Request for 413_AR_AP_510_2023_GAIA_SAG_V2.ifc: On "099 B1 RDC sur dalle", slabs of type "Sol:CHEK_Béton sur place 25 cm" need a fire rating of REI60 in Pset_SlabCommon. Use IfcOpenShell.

First a look at what the model holds.

```python
import ifcopenshell
import ifcopenshell.util.element

model = ifcopenshell.open("413_AR_AP_510_2023_GAIA_SAG_V2.ifc")
print(model.schema)
storey = next(s for s in model.by_type("IfcBuildingStorey") if s.Name == "099 B1 RDC sur dalle")
slabs = [e for e in ifcopenshell.util.element.get_decomposition(storey) if e.is_a("IfcSlab")]
seen = {}
for e in slabs:
    element_type = ifcopenshell.util.element.get_type(e)
    key = (element_type.Name if element_type != e and element_type else None, ifcopenshell.util.element.get_pset(e, "Pset_SlabCommon", "FireRating"))
    seen[key] = seen.get(key, 0) + 1
for (name, value), count in sorted(seen.items(), key=str):
    print(count, "x", name, "|", value)
```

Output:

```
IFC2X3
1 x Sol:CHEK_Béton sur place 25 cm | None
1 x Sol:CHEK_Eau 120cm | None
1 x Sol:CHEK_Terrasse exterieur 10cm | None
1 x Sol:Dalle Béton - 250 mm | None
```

```python
import ifcopenshell
import ifcopenshell.api.pset
import ifcopenshell.util.element

model = ifcopenshell.open("413_AR_AP_510_2023_GAIA_SAG_V2.ifc")

storey = next(s for s in model.by_type("IfcBuildingStorey") if s.Name == "099 B1 RDC sur dalle")
slabs = [e for e in ifcopenshell.util.element.get_decomposition(storey) if e.is_a("IfcSlab")]

count = 0
for e in slabs:
    element_type = ifcopenshell.util.element.get_type(e)
    if element_type in (None, e) or element_type.Name != "Sol:CHEK_Béton sur place 25 cm":
        continue
    # add_pset returns the element's existing set when there is one.
    pset = ifcopenshell.api.pset.add_pset(model, product=e, name="Pset_SlabCommon")
    ifcopenshell.api.pset.edit_pset(model, pset=pset, properties={"FireRating": "REI60"})
    count += 1

print(count, "slabs updated")

model.write("413_AR_AP_510_2023_GAIA_SAG_V2-out.ifc")
```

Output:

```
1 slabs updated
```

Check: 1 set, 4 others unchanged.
